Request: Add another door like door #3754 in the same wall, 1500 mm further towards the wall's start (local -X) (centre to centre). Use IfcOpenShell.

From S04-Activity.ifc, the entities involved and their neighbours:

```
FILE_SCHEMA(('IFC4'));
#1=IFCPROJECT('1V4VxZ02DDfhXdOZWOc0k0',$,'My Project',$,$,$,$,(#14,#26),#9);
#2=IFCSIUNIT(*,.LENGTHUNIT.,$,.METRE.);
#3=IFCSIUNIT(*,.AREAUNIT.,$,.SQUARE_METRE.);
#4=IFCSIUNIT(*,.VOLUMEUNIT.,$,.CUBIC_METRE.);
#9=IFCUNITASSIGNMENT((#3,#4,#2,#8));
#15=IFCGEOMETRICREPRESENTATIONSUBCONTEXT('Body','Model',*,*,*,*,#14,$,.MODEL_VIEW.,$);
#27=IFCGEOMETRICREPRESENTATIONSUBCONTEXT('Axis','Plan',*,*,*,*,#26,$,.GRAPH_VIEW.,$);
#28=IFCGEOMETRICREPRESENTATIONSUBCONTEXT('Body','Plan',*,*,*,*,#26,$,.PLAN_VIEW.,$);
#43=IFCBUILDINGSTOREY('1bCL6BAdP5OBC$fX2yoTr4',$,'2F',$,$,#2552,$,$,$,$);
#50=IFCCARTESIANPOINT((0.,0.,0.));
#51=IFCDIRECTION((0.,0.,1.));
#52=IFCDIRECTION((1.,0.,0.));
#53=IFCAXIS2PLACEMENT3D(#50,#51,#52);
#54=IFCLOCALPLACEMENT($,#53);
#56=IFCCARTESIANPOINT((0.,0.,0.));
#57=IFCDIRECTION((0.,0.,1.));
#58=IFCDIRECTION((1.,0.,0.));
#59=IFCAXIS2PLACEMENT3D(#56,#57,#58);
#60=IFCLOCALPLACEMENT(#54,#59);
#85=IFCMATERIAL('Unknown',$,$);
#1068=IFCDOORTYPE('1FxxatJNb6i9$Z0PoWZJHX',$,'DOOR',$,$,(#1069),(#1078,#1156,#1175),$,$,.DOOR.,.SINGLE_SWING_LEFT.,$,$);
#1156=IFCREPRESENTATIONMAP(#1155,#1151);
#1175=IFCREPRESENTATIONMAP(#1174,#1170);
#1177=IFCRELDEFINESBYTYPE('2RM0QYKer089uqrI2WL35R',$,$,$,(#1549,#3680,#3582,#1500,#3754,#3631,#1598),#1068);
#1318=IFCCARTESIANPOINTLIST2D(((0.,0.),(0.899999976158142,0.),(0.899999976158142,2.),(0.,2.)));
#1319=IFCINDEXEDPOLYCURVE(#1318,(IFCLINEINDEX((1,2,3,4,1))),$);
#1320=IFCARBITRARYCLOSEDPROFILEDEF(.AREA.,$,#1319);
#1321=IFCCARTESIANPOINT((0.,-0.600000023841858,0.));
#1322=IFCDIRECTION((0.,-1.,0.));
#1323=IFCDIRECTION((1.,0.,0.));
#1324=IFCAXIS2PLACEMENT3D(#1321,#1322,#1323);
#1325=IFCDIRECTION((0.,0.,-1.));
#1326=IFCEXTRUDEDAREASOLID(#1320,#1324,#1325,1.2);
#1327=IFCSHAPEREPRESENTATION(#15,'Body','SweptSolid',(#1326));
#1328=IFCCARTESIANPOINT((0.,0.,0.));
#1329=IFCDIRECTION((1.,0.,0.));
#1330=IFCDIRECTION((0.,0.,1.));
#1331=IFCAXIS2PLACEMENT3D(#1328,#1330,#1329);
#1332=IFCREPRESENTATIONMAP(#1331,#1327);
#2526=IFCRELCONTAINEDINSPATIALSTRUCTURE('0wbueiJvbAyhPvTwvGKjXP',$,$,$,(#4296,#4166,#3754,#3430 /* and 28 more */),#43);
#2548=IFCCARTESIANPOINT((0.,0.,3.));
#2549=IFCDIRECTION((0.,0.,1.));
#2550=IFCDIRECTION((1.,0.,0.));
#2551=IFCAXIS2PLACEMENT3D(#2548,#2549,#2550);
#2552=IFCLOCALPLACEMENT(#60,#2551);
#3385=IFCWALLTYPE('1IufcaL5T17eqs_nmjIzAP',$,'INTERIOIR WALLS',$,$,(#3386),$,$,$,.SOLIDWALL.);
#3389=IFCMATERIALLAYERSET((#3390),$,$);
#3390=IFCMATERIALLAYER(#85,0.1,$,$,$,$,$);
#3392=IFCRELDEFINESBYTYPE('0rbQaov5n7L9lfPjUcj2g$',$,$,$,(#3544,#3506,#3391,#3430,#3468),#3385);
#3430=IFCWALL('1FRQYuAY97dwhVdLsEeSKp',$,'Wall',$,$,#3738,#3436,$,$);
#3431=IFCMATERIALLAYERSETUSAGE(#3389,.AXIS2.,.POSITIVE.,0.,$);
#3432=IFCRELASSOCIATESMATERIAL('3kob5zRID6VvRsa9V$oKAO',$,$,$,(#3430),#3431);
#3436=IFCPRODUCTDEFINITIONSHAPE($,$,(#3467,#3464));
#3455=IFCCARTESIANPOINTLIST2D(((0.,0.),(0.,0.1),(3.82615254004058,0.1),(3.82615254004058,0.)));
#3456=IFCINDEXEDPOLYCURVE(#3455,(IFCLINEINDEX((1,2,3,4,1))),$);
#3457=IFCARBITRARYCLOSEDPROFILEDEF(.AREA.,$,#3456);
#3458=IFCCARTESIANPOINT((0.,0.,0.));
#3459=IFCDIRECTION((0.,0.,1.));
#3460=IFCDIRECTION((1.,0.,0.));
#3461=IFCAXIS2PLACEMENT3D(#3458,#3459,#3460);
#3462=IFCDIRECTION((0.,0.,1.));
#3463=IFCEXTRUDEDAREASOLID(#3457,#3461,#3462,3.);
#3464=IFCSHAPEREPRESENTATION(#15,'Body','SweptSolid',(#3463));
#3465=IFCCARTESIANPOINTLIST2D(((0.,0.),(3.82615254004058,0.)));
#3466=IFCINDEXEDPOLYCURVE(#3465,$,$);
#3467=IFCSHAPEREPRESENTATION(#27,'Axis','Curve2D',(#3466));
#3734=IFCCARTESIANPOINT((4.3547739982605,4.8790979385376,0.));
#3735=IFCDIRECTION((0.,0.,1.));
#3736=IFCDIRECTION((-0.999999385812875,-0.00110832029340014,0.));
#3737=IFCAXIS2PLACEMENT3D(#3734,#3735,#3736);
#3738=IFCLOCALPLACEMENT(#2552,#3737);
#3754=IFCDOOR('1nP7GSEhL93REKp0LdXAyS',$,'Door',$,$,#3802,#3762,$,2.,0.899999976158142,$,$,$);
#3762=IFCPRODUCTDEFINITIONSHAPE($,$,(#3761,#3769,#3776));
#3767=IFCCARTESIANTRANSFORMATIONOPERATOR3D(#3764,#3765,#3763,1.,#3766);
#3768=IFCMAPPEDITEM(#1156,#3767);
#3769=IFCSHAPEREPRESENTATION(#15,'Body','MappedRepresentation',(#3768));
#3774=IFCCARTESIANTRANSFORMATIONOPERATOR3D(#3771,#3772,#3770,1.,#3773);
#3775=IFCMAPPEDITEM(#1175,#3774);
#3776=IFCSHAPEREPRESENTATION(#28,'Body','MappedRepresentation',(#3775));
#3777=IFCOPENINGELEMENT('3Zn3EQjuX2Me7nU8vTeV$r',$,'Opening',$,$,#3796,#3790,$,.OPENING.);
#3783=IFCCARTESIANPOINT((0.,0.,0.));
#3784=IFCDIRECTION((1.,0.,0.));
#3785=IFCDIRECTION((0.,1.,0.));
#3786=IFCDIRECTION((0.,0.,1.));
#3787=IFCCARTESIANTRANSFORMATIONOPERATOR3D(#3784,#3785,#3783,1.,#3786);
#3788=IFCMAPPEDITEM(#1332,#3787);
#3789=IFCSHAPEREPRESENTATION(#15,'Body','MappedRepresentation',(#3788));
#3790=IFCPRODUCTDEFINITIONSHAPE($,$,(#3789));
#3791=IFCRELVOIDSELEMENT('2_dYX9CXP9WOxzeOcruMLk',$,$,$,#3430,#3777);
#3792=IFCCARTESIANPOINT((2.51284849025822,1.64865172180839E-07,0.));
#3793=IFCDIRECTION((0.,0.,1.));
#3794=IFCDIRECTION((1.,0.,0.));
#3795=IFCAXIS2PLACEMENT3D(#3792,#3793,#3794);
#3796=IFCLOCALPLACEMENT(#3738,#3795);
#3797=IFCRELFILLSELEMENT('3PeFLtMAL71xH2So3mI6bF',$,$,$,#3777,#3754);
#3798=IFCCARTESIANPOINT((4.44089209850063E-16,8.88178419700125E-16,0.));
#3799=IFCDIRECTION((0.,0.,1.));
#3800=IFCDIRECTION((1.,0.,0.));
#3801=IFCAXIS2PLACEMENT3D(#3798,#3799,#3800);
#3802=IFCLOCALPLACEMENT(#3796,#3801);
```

```python
import ifcopenshell
import ifcopenshell.api.feature
import ifcopenshell.api.geometry
import ifcopenshell.api.root
import ifcopenshell.geom
import ifcopenshell.util.element
import ifcopenshell.util.placement
import ifcopenshell.util.shape

model = ifcopenshell.open("S04-Activity.ifc")
settings = ifcopenshell.geom.settings()


def volume(element):
    """Net volume in cubic metres, openings subtracted."""
    shape = ifcopenshell.geom.create_shape(settings, element)
    return ifcopenshell.util.shape.get_volume(shape.geometry)


door = model.by_id(3754)
opening = door.FillsVoids[0].RelatingOpeningElement
wall = opening.VoidsElements[0].RelatingBuildingElement
before = volume(wall)
shift = ifcopenshell.util.placement.get_local_placement(wall.ObjectPlacement)[:3, 0] * -1.5

# copy_class copies the void relationship, type, container and properties, but no geometry.
new_opening = ifcopenshell.api.root.copy_class(model, product=opening)
new_opening.Representation = ifcopenshell.util.element.copy_deep(
    model, opening.Representation, exclude=["IfcGeometricRepresentationContext", "IfcRepresentationMap"]
)
new_door = ifcopenshell.api.root.copy_class(model, product=door)
new_door.Representation = ifcopenshell.util.element.copy_deep(
    model, door.Representation, exclude=["IfcGeometricRepresentationContext", "IfcRepresentationMap"]
)
ifcopenshell.api.feature.add_filling(model, opening=new_opening, element=new_door)

for old, new in ((opening, new_opening), (door, new_door)):
    matrix = ifcopenshell.util.placement.get_local_placement(old.ObjectPlacement)
    matrix[:3, 3] += shift
    ifcopenshell.api.geometry.edit_object_placement(model, product=new, matrix=matrix, is_si=False)

after = volume(wall)

print(f"wall volume {before:.3f} -> {after:.3f} m3")

model.write("S04-Activity_v2.ifc")
```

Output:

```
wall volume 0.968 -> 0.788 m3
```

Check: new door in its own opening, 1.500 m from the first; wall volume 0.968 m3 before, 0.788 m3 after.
